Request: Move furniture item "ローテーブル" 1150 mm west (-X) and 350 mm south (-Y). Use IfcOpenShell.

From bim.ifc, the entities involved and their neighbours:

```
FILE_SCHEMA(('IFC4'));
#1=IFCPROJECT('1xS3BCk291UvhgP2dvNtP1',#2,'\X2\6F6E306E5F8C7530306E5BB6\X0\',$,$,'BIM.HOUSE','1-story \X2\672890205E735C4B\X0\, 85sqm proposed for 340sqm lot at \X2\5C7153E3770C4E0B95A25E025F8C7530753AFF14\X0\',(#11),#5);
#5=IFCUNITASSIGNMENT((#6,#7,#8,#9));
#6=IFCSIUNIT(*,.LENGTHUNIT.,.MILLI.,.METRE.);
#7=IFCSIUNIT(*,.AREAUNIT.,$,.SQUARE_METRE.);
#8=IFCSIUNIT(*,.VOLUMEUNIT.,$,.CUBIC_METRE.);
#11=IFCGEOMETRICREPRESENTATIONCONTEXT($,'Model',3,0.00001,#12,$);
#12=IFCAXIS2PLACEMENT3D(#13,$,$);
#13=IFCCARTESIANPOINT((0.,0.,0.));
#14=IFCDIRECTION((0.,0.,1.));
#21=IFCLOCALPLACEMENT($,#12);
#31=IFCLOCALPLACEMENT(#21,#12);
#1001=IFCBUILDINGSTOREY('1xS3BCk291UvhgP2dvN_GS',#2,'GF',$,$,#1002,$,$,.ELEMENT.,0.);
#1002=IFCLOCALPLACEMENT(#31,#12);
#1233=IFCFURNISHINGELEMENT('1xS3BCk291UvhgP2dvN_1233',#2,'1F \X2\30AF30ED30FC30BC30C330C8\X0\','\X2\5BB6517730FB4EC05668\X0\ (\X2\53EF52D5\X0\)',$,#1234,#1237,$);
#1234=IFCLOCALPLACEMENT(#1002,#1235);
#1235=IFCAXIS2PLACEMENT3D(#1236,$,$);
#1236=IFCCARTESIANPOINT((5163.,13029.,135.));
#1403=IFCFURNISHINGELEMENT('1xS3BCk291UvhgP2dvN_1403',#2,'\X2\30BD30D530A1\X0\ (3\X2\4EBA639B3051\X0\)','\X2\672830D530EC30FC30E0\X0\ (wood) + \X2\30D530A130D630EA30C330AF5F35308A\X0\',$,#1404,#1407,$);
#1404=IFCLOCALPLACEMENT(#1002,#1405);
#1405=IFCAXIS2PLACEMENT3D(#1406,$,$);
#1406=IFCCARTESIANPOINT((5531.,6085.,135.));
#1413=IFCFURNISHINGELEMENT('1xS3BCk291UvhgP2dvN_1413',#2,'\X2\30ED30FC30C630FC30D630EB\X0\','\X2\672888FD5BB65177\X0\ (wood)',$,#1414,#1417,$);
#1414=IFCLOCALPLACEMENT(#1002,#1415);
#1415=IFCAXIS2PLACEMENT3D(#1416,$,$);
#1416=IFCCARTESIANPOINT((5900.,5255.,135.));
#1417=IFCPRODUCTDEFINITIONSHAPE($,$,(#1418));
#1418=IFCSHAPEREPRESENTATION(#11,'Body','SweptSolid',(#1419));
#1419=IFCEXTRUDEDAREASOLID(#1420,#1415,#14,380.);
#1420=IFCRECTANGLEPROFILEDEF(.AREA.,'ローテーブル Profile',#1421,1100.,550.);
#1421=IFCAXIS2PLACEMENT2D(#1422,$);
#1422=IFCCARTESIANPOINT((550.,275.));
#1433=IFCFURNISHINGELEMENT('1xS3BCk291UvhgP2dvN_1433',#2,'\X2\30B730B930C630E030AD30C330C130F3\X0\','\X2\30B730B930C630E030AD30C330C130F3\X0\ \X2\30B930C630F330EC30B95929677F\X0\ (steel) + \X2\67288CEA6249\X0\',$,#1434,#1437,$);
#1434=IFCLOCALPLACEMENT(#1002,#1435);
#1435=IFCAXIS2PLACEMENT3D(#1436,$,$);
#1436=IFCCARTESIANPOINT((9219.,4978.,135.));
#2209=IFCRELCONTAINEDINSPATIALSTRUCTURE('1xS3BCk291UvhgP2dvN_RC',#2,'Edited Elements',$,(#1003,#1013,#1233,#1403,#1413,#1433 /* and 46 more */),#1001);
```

```python
import ifcopenshell
import ifcopenshell.api.geometry
import ifcopenshell.util.placement
import ifcopenshell.util.unit

model = ifcopenshell.open("bim.ifc")
unit_scale = ifcopenshell.util.unit.calculate_unit_scale(model)

item = model.by_guid("1xS3BCk291UvhgP2dvN_1413")
matrix = ifcopenshell.util.placement.get_local_placement(item.ObjectPlacement)
matrix[0, 3] -= 1.15 / unit_scale
matrix[1, 3] -= 0.35 / unit_scale
ifcopenshell.api.geometry.edit_object_placement(model, product=item, matrix=matrix, is_si=False)

print(ifcopenshell.util.placement.get_local_placement(item.ObjectPlacement).round(3) + 0.0)

model.write("bim_updated.ifc")
```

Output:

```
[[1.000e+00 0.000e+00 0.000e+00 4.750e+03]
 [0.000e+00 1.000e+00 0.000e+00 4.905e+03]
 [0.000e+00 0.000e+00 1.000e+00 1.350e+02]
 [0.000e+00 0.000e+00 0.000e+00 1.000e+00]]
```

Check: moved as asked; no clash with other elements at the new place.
